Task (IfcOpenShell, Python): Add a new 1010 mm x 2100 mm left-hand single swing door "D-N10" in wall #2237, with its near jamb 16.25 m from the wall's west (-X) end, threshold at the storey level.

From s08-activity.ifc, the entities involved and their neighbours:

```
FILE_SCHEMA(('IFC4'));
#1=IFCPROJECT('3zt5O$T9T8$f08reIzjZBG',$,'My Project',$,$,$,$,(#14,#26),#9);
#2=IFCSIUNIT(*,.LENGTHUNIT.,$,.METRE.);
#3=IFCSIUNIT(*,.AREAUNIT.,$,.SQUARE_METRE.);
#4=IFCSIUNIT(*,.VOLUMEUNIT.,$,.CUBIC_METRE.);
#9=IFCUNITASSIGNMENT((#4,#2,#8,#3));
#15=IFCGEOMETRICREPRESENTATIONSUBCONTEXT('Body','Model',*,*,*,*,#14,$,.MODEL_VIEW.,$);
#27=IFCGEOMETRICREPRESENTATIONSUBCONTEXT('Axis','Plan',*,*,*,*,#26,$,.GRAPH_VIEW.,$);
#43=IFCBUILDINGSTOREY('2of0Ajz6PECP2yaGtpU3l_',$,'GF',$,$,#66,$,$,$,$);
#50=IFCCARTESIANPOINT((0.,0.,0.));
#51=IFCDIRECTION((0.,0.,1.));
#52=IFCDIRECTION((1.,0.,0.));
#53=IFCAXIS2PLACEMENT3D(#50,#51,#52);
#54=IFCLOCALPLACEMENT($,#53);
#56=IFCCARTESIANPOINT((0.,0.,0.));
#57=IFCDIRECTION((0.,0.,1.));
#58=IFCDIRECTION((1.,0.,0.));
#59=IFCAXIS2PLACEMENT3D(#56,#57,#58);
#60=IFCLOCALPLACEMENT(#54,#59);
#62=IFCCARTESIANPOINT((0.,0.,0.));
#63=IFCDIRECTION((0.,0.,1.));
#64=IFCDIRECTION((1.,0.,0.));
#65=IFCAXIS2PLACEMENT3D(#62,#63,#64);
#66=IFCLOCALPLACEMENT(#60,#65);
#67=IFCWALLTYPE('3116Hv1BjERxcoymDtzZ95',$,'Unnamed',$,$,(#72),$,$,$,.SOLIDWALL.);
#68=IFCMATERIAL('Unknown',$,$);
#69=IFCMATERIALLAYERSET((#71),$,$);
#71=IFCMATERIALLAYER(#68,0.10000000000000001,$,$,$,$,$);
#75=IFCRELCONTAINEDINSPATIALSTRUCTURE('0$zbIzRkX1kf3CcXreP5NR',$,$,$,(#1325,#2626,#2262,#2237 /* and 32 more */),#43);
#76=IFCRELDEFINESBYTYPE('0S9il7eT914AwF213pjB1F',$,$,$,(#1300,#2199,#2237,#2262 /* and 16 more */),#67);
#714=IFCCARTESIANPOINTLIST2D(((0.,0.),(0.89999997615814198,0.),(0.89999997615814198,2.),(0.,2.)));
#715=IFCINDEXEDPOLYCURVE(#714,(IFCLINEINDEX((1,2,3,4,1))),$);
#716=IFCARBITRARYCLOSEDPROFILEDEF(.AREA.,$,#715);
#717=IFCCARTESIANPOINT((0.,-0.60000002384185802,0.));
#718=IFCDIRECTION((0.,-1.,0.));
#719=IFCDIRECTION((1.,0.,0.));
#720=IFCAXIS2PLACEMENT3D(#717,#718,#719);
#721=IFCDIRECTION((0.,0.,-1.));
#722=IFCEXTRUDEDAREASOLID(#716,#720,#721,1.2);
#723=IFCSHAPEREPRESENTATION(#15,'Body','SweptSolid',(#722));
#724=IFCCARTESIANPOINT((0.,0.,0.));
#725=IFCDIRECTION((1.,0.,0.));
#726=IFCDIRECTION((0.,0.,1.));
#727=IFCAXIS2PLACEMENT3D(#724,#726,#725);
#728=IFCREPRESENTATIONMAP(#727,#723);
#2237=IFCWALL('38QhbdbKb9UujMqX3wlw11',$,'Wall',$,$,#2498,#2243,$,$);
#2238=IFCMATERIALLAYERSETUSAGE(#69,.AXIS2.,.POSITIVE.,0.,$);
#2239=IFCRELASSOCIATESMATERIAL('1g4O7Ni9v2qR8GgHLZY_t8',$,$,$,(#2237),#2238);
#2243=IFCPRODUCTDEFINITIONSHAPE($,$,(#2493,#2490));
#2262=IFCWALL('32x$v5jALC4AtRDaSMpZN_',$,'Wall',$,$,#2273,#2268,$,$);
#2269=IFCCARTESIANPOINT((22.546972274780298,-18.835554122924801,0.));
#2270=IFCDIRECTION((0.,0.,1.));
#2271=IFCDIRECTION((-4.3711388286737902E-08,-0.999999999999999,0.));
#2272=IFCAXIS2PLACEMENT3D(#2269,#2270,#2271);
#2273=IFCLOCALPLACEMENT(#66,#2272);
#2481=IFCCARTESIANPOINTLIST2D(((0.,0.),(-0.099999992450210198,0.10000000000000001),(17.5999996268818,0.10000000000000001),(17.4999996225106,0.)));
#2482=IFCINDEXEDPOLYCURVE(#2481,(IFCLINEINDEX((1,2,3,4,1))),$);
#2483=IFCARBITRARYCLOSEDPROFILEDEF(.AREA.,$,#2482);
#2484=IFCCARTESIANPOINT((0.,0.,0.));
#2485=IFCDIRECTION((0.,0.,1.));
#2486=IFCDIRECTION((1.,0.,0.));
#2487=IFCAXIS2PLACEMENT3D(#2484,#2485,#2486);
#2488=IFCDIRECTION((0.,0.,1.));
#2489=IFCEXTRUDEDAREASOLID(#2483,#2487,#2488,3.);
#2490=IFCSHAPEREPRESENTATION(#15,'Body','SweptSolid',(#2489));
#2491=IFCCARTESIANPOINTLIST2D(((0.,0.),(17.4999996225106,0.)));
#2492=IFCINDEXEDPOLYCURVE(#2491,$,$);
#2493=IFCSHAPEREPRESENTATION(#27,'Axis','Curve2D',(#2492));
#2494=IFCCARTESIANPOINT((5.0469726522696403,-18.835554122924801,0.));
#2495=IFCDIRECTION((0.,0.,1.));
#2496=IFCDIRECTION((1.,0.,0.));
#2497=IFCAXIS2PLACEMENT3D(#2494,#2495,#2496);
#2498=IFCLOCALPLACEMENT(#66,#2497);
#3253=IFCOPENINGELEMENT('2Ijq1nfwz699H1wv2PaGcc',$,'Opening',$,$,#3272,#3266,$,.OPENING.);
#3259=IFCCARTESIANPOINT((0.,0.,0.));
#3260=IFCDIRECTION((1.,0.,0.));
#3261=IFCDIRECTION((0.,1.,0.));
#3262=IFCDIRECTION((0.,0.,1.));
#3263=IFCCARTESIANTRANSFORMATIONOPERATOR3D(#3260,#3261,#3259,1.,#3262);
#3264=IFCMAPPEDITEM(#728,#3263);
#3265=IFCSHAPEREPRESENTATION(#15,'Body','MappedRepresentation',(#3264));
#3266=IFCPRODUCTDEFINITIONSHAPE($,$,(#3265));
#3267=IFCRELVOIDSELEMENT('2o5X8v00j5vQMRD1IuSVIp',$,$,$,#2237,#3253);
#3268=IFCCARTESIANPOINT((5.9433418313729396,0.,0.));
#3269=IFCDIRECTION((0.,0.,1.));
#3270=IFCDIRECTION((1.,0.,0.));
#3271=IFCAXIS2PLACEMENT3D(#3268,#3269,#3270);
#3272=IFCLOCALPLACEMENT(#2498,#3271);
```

```python
import numpy as np
import ifcopenshell
import ifcopenshell.api.feature
import ifcopenshell.api.geometry
import ifcopenshell.api.root
import ifcopenshell.api.spatial
import ifcopenshell.geom
import ifcopenshell.util.element
import ifcopenshell.util.placement
import ifcopenshell.util.representation
import ifcopenshell.util.shape
import ifcopenshell.util.unit

model = ifcopenshell.open("s08-activity.ifc")
unit_scale = ifcopenshell.util.unit.calculate_unit_scale(model)
settings = ifcopenshell.geom.settings()


def volume(element):
    """Net volume in cubic metres, openings subtracted."""
    shape = ifcopenshell.geom.create_shape(settings, element)
    return ifcopenshell.util.shape.get_volume(shape.geometry)


wall = model.by_guid("38QhbdbKb9UujMqX3wlw11")
storey = ifcopenshell.util.element.get_container(wall, ifc_class="IfcBuildingStorey")
context = ifcopenshell.util.representation.get_context(model, "Model", "Body", "MODEL_VIEW")
before = volume(wall)

width, height, from_end, sill = 1.01, 2.1, 16.25, 0.0  # metres

# The wall runs along its own X axis, and the end named is its -X end.
wall_shape = ifcopenshell.geom.create_shape(settings, wall)
x, y, z = ifcopenshell.util.shape.get_vertices(wall_shape.geometry).T
start = x.min() + from_end
face, thickness = float(y.min()), float(y.max() - y.min())
wall_matrix = ifcopenshell.util.placement.get_local_placement(wall.ObjectPlacement)
level = ifcopenshell.util.placement.get_local_placement(storey.ObjectPlacement)[2, 3]


def in_wall(x, y):
    """Placement at x, y metres in the wall's axes, at sill height."""
    matrix = wall_matrix.copy()
    matrix[:, 3] = wall_matrix @ np.array([x / unit_scale, y / unit_scale, 0.0, 1.0])
    matrix[2, 3] = level + sill / unit_scale
    return matrix


# Opening: a box that overshoots both wall faces by 50 mm.
opening = ifcopenshell.api.root.create_entity(model, ifc_class="IfcOpeningElement", predefined_type="OPENING")
box = ifcopenshell.api.geometry.add_wall_representation(
    model, context=context, length=width, height=height, thickness=thickness + 0.1
)
ifcopenshell.api.geometry.assign_representation(model, product=opening, representation=box)
ifcopenshell.api.geometry.edit_object_placement(model, product=opening, matrix=in_wall(start, face - 0.05), is_si=False)
ifcopenshell.api.feature.add_feature(model, feature=opening, element=wall)

door = ifcopenshell.api.root.create_entity(model, ifc_class="IfcDoor", name="D-N10", predefined_type="DOOR")
door.OverallWidth, door.OverallHeight = width / unit_scale, height / unit_scale
door.OperationType = "SINGLE_SWING_LEFT"
body = ifcopenshell.api.geometry.add_door_representation(
    model,
    context=context,
    overall_width=door.OverallWidth,
    overall_height=door.OverallHeight,
    operation_type="SINGLE_SWING_LEFT",
    lining_properties={"LiningDepth": thickness / unit_scale, "ThresholdDepth": thickness / unit_scale},
)
ifcopenshell.api.geometry.assign_representation(model, product=door, representation=body)
ifcopenshell.api.spatial.assign_container(model, products=[door], relating_structure=storey)
ifcopenshell.api.feature.add_filling(model, opening=opening, element=door)

# The lining spans the wall, so the door starts at the wall face.
ifcopenshell.api.geometry.edit_object_placement(model, product=door, matrix=in_wall(start, face), is_si=False)

after = volume(wall)

print(f"wall volume {before:.3f} -> {after:.3f} m3")

model.write("s08-activity_updated.ifc")
```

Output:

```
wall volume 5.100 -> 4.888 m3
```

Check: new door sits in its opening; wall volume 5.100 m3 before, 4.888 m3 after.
